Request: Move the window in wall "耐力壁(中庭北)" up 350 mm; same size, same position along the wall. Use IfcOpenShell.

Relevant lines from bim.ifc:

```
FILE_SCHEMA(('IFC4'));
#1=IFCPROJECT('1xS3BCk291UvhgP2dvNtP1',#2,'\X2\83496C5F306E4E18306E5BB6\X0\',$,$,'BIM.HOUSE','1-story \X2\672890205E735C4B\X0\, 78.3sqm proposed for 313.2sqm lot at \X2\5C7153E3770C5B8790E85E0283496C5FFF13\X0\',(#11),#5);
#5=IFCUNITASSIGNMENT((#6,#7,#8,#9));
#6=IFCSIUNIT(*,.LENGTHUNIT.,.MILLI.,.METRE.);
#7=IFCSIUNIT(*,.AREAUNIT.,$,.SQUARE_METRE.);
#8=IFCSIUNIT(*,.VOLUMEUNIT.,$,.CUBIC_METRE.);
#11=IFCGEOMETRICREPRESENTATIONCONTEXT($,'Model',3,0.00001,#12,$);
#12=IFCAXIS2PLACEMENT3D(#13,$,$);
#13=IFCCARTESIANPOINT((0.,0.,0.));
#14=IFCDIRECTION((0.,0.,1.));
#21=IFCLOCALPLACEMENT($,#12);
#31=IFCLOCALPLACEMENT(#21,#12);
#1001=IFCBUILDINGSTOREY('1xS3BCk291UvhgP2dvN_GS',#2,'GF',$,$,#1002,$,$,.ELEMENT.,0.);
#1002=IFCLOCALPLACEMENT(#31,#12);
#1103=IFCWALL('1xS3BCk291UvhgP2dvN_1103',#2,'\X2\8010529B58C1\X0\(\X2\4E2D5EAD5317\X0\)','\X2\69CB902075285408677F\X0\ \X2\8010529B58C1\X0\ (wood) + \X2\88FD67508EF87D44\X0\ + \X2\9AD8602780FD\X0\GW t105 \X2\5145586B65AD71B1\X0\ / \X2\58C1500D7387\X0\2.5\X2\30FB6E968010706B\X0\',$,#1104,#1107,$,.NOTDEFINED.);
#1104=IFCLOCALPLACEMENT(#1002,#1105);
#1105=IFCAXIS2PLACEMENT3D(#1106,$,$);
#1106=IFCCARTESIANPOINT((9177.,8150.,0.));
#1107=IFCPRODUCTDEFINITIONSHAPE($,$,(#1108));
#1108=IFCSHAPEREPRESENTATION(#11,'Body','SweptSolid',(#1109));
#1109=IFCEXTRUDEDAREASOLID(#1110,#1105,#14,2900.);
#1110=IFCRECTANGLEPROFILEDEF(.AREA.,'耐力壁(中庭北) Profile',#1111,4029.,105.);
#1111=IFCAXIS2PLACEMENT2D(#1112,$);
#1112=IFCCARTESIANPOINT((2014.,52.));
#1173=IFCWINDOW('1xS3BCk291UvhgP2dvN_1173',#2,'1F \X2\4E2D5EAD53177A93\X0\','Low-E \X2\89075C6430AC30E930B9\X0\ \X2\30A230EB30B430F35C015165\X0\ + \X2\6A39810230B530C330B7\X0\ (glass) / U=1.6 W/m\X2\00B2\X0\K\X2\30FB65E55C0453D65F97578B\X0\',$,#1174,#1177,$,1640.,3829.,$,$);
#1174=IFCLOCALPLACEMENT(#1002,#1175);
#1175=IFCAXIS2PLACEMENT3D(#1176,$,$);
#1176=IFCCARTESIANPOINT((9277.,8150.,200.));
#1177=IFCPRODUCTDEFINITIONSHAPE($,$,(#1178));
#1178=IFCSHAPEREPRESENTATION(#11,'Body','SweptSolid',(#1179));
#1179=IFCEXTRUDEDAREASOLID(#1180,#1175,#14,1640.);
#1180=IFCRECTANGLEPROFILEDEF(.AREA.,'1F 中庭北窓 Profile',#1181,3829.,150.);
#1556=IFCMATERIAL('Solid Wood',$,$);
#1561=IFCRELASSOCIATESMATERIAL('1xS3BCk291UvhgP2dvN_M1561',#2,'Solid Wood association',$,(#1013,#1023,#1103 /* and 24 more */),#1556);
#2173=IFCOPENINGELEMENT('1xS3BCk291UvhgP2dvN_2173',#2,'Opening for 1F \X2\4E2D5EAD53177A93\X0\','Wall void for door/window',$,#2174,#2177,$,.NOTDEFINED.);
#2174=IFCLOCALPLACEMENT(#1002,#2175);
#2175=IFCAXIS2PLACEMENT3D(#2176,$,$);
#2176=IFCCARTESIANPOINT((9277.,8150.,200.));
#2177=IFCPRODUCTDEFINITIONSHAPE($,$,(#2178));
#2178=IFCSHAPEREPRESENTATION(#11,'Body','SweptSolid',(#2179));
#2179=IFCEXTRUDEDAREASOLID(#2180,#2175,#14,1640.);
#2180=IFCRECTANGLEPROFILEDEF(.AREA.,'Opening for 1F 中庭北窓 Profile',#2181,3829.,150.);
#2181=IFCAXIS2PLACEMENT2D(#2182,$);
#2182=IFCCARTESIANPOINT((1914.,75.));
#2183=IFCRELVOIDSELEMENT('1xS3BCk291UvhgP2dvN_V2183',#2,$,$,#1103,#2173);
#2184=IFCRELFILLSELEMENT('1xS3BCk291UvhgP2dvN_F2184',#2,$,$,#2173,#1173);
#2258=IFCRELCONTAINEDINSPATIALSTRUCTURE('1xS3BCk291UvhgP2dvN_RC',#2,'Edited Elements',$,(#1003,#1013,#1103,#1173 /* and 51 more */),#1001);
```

```python
import numpy as np
import ifcopenshell
import ifcopenshell.api.geometry
import ifcopenshell.util.placement
import ifcopenshell.util.unit

model = ifcopenshell.open("bim.ifc")
unit_scale = ifcopenshell.util.unit.calculate_unit_scale(model)

window = model.by_guid("1xS3BCk291UvhgP2dvN_1173")
opening = window.FillsVoids[0].RelatingOpeningElement
dz = 350.0

shift = np.array([0.0, 0.0, dz])
# The window is not placed relative to its opening, so move both.
for product in (opening, window):
    matrix = ifcopenshell.util.placement.get_local_placement(product.ObjectPlacement)
    matrix[:3, 3] += shift
    ifcopenshell.api.geometry.edit_object_placement(model, product=product, matrix=matrix, is_si=False)

print(f"moved by {dz * unit_scale:+.3f} m")

model.write("bim_updated.ifc")
```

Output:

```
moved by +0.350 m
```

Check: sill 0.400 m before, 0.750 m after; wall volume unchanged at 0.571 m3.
